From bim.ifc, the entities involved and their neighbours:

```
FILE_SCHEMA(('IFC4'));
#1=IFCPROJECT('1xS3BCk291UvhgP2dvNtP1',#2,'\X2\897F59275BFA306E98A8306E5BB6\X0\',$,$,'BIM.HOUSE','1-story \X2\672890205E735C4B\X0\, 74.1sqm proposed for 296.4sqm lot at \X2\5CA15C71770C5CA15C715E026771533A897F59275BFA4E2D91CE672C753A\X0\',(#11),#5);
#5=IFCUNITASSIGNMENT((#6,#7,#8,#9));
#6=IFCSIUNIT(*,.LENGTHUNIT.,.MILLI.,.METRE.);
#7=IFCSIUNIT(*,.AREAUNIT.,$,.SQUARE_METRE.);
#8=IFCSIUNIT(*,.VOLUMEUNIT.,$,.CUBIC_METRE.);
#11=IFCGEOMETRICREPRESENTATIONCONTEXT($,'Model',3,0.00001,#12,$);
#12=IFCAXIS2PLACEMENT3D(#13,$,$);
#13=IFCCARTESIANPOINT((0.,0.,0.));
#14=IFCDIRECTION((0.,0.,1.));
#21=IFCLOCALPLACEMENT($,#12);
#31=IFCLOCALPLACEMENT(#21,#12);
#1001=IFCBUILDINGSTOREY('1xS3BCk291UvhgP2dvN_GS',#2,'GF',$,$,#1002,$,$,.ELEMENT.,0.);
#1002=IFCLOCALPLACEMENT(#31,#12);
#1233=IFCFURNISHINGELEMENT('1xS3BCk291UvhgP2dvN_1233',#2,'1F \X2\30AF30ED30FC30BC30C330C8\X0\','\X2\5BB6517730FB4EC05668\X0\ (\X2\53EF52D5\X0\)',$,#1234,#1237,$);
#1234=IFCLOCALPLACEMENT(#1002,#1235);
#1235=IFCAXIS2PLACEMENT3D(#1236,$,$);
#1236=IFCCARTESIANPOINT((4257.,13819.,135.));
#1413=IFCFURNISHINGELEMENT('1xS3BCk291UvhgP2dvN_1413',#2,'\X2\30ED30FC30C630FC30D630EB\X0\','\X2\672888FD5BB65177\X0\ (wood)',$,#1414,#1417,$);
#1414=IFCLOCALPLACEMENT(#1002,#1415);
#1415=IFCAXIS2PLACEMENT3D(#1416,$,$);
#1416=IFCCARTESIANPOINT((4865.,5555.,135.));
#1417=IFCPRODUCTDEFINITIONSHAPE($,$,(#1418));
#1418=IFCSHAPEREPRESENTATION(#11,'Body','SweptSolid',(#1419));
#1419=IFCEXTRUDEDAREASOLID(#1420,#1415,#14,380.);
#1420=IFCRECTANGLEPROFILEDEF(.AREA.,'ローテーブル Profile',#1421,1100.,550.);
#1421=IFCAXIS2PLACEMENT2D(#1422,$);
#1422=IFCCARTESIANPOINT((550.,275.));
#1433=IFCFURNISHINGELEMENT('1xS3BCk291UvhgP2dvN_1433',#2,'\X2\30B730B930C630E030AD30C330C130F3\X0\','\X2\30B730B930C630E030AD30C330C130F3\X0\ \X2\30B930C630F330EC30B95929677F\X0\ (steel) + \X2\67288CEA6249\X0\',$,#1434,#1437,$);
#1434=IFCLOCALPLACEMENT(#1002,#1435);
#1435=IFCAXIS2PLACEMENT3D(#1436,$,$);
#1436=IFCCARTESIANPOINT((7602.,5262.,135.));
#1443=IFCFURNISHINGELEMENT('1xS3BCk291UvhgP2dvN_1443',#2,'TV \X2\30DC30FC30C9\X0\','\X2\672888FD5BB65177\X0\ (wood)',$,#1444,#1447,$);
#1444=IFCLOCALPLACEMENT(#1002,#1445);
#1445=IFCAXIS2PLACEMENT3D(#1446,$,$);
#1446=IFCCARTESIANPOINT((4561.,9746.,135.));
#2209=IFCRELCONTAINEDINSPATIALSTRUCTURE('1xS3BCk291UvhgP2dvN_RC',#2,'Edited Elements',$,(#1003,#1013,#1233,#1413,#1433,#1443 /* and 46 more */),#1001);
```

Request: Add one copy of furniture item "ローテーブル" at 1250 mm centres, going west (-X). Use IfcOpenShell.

```python
import numpy as np
import ifcopenshell
import ifcopenshell.api.geometry
import ifcopenshell.api.root
import ifcopenshell.util.element
import ifcopenshell.util.placement
import ifcopenshell.util.unit

model = ifcopenshell.open("bim.ifc")
unit_scale = ifcopenshell.util.unit.calculate_unit_scale(model)


def reuse_history(source, copy):
    """copy_class also copies each property set's owner history, people and application; keep the originals."""
    for rel in copy.IsDefinedBy:
        if rel.is_a("IfcRelDefinesByProperties") and (history := rel.RelatingPropertyDefinition.OwnerHistory):
            rel.RelatingPropertyDefinition.OwnerHistory = source.OwnerHistory
            ifcopenshell.util.element.remove_deep2(model, history)


source = model.by_guid("1xS3BCk291UvhgP2dvN_1413")
base = ifcopenshell.util.placement.get_local_placement(source.ObjectPlacement)
step = np.array([-1.0, 0.0, 0.0]) * 1.25 / unit_scale

for i in range(1, 2):
    copy = ifcopenshell.api.root.copy_class(model, product=source)
    copy.Representation = ifcopenshell.util.element.copy_deep(
        model, source.Representation, exclude=["IfcGeometricRepresentationContext", "IfcRepresentationMap"]
    )
    reuse_history(source, copy)
    matrix = base.copy()
    matrix[:3, 3] += i * step
    print("added at", matrix[:3, 3].round(3) + 0.0)
    ifcopenshell.api.geometry.edit_object_placement(model, product=copy, matrix=matrix, is_si=False)

model.write("bim_rev.ifc")
```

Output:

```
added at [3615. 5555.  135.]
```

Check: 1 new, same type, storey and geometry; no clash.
